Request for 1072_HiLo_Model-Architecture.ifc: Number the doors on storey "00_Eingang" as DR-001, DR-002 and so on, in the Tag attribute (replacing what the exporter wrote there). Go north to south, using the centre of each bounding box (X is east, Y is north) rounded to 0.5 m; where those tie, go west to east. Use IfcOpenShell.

First a look at what the model holds.

```python
import ifcopenshell
import ifcopenshell.util.element
import ifcopenshell.util.placement

model = ifcopenshell.open("1072_HiLo_Model-Architecture.ifc")
print(model.schema)
storey = next(s for s in model.by_type("IfcBuildingStorey") if s.Name == "00_Eingang")
doors = [e for e in ifcopenshell.util.element.get_decomposition(storey) if e.is_a("IfcDoor")]
for e in sorted(doors, key=lambda e: e.id()):
    origin = ifcopenshell.util.placement.get_local_placement(e.ObjectPlacement)[:3, 3]
    print(e.id(), e.Tag, e.Name, origin.round(2) + 0.0, sep=" | ")
```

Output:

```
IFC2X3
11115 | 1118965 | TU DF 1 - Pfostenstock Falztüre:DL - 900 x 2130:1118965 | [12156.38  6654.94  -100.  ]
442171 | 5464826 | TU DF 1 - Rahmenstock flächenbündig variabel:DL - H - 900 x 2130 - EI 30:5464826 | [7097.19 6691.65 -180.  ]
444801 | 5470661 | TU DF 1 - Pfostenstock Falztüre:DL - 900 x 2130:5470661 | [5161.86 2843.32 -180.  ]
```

```python
import ifcopenshell
import ifcopenshell.geom
import ifcopenshell.util.element
import ifcopenshell.util.shape

model = ifcopenshell.open("1072_HiLo_Model-Architecture.ifc")
settings = ifcopenshell.geom.settings()
settings.set("use-world-coords", True)


def centre(element):
    shape = ifcopenshell.geom.create_shape(settings, element)
    return ifcopenshell.util.shape.get_bbox_centroid(shape.geometry)


storey = next(s for s in model.by_type("IfcBuildingStorey") if s.Name == "00_Eingang")
doors = [e for e in ifcopenshell.util.element.get_decomposition(storey) if e.is_a("IfcDoor")]

# Insertion points can sit at a corner or the storey origin, so sort by the geometry (in metres).
centres = {e: centre(e) for e in doors}
doors.sort(key=lambda e: (-round(centres[e][1] / 0.5), centres[e][0]))

for i, e in enumerate(doors, start=1):
    number = f"DR-0{i:02d}"
    e.Tag = number
    print(e.id(), number)

model.write("1072_HiLo_Model-Architecture_rev.ifc")
```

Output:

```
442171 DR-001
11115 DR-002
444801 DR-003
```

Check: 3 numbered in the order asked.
